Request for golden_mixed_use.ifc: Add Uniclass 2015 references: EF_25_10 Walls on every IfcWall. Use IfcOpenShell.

First a look at what the model holds.

```python
import ifcopenshell

model = ifcopenshell.open("golden_mixed_use.ifc")
print(model.schema)
print("classifications:", [c.Name for c in model.by_type("IfcClassification")])
for ifc_class in ("IfcDoor", "IfcRoof", "IfcStair", "IfcWall", "IfcWindow"):
    print(ifc_class, len(model.by_type(ifc_class)))
```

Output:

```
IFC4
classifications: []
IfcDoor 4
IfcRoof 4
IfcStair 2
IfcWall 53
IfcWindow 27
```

```python
import ifcopenshell
import ifcopenshell.api.classification

model = ifcopenshell.open("golden_mixed_use.ifc")

system = ifcopenshell.api.classification.add_classification(model, classification="Uniclass 2015")

codes = {
    "IfcWall": ("EF_25_10", "Walls"),
}
for ifc_class, (code, name) in codes.items():
    products = model.by_type(ifc_class)
    ifcopenshell.api.classification.add_reference(
        model, products=products, classification=system, identification=code, name=name
    )
    print(code, len(products))

model.write("golden_mixed_use_rev.ifc")
```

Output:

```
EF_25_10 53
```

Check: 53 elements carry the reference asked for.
